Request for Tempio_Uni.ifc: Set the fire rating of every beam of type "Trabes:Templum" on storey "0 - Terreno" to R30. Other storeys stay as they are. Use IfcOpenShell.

First a look at what the model holds.

```python
import ifcopenshell
import ifcopenshell.util.element

model = ifcopenshell.open("Tempio_Uni.ifc")
print(model.schema)
storey = next(s for s in model.by_type("IfcBuildingStorey") if s.Name == "0 - Terreno")
beams = [e for e in ifcopenshell.util.element.get_decomposition(storey) if e.is_a("IfcBeam")]
seen = {}
for e in beams:
    element_type = ifcopenshell.util.element.get_type(e)
    key = (element_type.Name if element_type != e and element_type else None, ifcopenshell.util.element.get_pset(e, "Pset_BeamCommon", "FireRating"))
    seen[key] = seen.get(key, 0) + 1
for (name, value), count in sorted(seen.items(), key=str):
    print(count, "x", name, "|", value)
```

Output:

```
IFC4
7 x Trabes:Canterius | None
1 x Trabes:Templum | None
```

```python
import ifcopenshell
import ifcopenshell.api.pset
import ifcopenshell.util.element

model = ifcopenshell.open("Tempio_Uni.ifc")

storey = next(s for s in model.by_type("IfcBuildingStorey") if s.Name == "0 - Terreno")
beams = [e for e in ifcopenshell.util.element.get_decomposition(storey) if e.is_a("IfcBeam")]

count = 0
for e in beams:
    element_type = ifcopenshell.util.element.get_type(e)
    if element_type in (None, e) or element_type.Name != "Trabes:Templum":
        continue
    # add_pset returns the element's existing set when there is one.
    pset = ifcopenshell.api.pset.add_pset(model, product=e, name="Pset_BeamCommon")
    ifcopenshell.api.pset.edit_pset(model, pset=pset, properties={"FireRating": "R30"})
    count += 1

print(count, "beams updated")

model.write("Tempio_Uni_rev.ifc")
```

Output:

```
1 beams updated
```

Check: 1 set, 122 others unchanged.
